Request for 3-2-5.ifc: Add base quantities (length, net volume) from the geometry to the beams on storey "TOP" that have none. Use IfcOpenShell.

First a look at what the model holds.

```python
import ifcopenshell
import ifcopenshell.util.element
import ifcopenshell.util.unit

model = ifcopenshell.open("3-2-5.ifc")
print(model.schema)
for unit_type in ("LENGTHUNIT", "AREAUNIT", "VOLUMEUNIT"):
    print(unit_type, ifcopenshell.util.unit.calculate_unit_scale(model, unit_type))
storey = next(s for s in model.by_type("IfcBuildingStorey") if s.Name == "TOP")
beams = [e for e in ifcopenshell.util.element.get_decomposition(storey) if e.is_a("IfcBeam")]
for e in sorted(beams, key=lambda e: e.id()):
    print(e.id(), e.is_a(), e.Name, list(ifcopenshell.util.element.get_psets(e, qtos_only=True)), sep=" | ")
```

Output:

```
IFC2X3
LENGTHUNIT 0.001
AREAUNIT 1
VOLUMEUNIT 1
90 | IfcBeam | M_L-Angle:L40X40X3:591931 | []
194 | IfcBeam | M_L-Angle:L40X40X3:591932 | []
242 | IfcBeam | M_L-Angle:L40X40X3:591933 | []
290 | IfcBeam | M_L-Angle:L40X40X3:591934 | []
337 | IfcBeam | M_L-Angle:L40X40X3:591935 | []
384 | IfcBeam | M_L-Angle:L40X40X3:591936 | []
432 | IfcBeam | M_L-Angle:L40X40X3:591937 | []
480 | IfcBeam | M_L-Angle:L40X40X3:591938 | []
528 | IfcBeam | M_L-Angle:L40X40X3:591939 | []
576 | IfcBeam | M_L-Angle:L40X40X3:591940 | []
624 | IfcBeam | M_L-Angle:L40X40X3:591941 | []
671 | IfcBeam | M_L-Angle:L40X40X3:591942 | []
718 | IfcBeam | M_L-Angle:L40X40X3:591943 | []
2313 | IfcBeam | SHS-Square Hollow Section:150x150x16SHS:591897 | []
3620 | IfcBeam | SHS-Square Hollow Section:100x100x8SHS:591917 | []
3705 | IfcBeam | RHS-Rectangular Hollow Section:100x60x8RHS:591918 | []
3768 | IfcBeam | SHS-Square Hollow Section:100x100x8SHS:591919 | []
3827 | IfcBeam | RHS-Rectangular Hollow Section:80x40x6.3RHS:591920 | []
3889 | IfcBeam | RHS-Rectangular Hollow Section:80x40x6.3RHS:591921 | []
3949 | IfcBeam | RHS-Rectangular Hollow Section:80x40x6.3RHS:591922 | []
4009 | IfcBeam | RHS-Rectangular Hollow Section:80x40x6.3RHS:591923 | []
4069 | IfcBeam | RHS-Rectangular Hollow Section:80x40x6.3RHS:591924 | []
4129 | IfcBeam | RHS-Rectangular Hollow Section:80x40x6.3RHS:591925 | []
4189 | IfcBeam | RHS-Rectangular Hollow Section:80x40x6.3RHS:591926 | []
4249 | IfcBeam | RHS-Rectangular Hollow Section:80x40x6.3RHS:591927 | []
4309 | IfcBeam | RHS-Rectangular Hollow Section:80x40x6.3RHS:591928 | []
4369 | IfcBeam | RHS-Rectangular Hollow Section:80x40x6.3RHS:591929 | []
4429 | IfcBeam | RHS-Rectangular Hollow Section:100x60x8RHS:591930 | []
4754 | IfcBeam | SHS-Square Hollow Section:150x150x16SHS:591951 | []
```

```python
import ifcopenshell
import ifcopenshell.api.pset
import ifcopenshell.geom
import ifcopenshell.util.element
import ifcopenshell.util.shape
import ifcopenshell.util.unit

model = ifcopenshell.open("3-2-5.ifc")
unit_scale = ifcopenshell.util.unit.calculate_unit_scale(model)
volume_scale = ifcopenshell.util.unit.calculate_unit_scale(model, "VOLUMEUNIT")
settings = ifcopenshell.geom.settings()

storey = next(s for s in model.by_type("IfcBuildingStorey") if s.Name == "TOP")
beams = [e for e in ifcopenshell.util.element.get_decomposition(storey) if e.is_a("IfcBeam")]

for e in sorted(beams, key=lambda e: e.id()):
    if ifcopenshell.util.element.get_psets(e, qtos_only=True, should_inherit=False):
        continue
    # Geometry comes back in metres, in the element's own axes.
    shape = ifcopenshell.geom.create_shape(settings, e)
    values = {
        "Length": ifcopenshell.util.shape.get_max_xyz(shape.geometry) / unit_scale,
        "NetVolume": ifcopenshell.util.shape.get_volume(shape.geometry) / volume_scale,
    }
    qto = ifcopenshell.api.pset.add_qto(model, product=e, name="BaseQuantities")
    ifcopenshell.api.pset.edit_qto(model, qto=qto, properties=values)
    print(e.id(), {k: round(v, 3) for k, v in values.items()})

model.write("3-2-5-out.ifc")
```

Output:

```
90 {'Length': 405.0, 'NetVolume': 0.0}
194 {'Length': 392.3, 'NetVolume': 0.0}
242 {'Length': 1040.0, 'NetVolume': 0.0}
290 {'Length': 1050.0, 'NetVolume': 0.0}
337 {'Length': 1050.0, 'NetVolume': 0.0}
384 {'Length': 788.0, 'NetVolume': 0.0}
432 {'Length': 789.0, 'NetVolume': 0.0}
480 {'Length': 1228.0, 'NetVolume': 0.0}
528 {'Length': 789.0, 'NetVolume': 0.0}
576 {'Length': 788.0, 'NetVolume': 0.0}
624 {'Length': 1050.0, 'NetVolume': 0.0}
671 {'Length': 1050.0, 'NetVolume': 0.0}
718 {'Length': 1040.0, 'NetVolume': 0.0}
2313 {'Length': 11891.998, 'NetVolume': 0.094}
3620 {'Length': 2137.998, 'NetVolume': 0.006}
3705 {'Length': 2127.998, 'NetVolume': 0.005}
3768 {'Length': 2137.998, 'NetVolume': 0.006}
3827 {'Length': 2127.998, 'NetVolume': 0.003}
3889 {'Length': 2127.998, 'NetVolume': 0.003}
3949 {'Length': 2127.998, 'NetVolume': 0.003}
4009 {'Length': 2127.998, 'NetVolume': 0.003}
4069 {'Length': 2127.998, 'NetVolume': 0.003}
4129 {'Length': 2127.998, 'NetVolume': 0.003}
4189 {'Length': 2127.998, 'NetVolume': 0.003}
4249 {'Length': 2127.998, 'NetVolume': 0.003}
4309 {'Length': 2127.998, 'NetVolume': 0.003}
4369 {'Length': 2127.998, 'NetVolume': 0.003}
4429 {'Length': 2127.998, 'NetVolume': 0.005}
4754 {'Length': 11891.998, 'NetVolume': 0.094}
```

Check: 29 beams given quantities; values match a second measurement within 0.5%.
